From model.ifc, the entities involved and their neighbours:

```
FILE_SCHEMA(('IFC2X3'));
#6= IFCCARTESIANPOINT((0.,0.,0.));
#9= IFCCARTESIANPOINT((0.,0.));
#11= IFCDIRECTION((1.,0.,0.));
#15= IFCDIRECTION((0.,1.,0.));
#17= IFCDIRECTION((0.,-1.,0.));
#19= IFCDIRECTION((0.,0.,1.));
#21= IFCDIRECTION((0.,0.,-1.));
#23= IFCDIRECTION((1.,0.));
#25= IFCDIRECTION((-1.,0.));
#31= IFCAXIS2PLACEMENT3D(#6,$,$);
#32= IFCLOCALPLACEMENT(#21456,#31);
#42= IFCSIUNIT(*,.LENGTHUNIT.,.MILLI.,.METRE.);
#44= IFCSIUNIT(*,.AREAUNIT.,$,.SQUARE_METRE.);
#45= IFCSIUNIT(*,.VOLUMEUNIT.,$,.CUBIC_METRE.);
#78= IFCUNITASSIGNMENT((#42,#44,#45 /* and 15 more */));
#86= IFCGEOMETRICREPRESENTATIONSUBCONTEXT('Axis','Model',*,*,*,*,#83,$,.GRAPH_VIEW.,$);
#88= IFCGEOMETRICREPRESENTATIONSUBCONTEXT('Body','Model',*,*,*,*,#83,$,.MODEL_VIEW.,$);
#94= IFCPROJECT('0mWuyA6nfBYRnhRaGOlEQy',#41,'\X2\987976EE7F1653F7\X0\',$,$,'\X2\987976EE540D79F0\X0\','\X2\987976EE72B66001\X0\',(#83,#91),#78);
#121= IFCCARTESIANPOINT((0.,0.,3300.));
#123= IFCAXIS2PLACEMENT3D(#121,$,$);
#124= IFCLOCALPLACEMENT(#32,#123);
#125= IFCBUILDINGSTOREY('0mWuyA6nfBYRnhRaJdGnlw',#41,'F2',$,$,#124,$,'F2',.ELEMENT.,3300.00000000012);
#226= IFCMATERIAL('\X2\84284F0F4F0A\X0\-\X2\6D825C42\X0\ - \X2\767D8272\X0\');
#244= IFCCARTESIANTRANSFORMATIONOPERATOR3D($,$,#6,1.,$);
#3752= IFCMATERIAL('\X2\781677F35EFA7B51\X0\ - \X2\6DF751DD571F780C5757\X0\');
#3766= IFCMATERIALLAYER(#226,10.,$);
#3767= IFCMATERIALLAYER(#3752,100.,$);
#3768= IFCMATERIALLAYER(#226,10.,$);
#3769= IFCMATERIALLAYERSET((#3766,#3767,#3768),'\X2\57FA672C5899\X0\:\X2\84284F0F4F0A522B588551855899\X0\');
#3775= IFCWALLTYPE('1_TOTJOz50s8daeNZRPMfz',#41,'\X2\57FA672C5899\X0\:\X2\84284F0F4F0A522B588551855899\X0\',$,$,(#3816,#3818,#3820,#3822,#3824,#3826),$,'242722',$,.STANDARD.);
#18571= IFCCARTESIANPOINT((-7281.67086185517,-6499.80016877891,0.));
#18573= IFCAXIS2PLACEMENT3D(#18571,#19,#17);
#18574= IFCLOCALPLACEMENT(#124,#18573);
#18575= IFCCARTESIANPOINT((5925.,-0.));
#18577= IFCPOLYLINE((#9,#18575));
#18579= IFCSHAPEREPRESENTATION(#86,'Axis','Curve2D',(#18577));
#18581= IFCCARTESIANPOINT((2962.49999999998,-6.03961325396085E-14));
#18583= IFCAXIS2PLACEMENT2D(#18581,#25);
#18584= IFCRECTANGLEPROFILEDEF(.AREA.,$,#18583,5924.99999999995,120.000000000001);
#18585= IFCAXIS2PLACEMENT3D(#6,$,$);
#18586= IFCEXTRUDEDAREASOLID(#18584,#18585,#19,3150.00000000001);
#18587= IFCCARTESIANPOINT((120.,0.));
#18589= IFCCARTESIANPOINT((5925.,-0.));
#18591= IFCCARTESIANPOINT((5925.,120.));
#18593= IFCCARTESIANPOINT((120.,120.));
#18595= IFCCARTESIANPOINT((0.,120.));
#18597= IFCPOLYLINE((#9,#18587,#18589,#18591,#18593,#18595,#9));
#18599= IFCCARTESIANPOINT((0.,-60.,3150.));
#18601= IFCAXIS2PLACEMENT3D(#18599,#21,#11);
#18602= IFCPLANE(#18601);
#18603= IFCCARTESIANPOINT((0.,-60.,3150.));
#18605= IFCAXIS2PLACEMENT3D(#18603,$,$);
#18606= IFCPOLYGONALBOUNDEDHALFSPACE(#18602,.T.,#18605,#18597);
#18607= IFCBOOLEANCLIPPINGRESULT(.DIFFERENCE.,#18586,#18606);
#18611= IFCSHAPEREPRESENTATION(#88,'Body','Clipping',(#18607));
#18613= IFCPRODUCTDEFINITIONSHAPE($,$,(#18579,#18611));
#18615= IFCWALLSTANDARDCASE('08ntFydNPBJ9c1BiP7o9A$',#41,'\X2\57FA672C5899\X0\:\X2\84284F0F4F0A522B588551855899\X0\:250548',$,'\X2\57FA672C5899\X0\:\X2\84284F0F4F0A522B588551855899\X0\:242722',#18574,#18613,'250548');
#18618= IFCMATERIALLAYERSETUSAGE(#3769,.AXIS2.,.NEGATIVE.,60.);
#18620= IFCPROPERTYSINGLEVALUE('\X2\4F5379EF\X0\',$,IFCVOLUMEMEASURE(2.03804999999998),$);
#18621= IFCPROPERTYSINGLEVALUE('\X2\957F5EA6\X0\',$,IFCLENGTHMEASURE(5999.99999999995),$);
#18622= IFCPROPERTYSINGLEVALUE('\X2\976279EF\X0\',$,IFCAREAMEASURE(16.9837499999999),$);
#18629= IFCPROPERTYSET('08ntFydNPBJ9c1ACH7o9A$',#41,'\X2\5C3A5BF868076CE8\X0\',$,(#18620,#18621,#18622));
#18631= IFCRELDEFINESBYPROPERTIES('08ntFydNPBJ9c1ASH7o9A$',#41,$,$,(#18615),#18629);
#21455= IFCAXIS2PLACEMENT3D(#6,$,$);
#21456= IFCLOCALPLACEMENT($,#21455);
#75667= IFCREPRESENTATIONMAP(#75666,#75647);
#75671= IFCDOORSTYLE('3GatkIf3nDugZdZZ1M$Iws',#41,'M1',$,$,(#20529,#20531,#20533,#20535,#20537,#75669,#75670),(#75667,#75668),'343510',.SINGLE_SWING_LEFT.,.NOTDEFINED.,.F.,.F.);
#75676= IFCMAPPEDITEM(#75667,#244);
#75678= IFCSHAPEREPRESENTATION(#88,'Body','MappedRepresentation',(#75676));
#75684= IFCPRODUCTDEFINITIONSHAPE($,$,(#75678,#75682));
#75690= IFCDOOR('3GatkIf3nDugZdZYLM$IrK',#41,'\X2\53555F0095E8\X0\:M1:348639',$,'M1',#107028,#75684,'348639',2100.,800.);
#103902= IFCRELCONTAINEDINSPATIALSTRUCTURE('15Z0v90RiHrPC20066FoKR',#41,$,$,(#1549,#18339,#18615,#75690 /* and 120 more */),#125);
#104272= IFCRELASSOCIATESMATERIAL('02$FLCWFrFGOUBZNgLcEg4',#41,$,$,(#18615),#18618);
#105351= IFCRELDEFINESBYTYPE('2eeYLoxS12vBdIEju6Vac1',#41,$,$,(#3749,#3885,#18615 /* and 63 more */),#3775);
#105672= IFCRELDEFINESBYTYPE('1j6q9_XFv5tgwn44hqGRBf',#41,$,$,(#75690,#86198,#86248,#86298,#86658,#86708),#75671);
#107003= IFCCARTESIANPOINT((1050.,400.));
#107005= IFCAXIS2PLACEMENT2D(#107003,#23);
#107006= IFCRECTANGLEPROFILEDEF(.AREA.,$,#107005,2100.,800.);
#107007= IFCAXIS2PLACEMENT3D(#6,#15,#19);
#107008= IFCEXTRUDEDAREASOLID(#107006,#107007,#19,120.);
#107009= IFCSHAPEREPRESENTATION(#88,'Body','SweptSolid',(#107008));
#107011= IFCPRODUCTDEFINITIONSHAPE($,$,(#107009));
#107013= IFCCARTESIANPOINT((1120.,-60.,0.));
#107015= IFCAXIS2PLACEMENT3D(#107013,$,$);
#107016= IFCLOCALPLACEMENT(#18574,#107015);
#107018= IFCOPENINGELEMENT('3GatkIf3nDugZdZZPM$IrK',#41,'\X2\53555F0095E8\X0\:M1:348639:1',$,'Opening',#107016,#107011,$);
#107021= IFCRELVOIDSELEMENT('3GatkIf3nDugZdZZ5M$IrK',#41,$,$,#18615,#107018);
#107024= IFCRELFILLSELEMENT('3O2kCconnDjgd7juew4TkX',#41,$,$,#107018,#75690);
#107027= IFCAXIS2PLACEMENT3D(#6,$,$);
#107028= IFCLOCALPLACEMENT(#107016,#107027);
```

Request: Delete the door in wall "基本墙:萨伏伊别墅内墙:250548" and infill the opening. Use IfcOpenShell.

```python
import ifcopenshell
import ifcopenshell.api.feature
import ifcopenshell.api.pset
import ifcopenshell.api.root
import ifcopenshell.geom
import ifcopenshell.util.element
import ifcopenshell.util.shape
import ifcopenshell.util.unit

model = ifcopenshell.open("model.ifc")
area_scale = ifcopenshell.util.unit.calculate_unit_scale(model, "AREAUNIT")
volume_scale = ifcopenshell.util.unit.calculate_unit_scale(model, "VOLUMEUNIT")
settings = ifcopenshell.geom.settings()


def volume(element):
    """Net volume in cubic metres, openings subtracted."""
    shape = ifcopenshell.geom.create_shape(settings, element)
    return ifcopenshell.util.shape.get_volume(shape.geometry)


door = model.by_id(75690)
opening = door.FillsVoids[0].RelatingOpeningElement
wall = opening.VoidsElements[0].RelatingBuildingElement
before = volume(wall)

ifcopenshell.api.root.remove_product(model, product=door)
ifcopenshell.api.feature.remove_feature(model, feature=opening)

after = volume(wall)
thickness = 0.12  # wall thickness in metres

# Update the wall's stored quantities.
pset = model.by_id(ifcopenshell.util.element.get_pset(wall, "尺寸标注", should_inherit=False)["id"])
ifcopenshell.api.pset.edit_pset(model, pset=pset, properties={
    "体积": model.create_entity("IfcVolumeMeasure", after / volume_scale),
    "面积": model.create_entity("IfcAreaMeasure", after / thickness / area_scale),
})

print(f"wall volume {before:.3f} -> {after:.3f} m3")

model.write("model-out.ifc")
```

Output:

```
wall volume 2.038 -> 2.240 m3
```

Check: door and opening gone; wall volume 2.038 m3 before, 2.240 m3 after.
